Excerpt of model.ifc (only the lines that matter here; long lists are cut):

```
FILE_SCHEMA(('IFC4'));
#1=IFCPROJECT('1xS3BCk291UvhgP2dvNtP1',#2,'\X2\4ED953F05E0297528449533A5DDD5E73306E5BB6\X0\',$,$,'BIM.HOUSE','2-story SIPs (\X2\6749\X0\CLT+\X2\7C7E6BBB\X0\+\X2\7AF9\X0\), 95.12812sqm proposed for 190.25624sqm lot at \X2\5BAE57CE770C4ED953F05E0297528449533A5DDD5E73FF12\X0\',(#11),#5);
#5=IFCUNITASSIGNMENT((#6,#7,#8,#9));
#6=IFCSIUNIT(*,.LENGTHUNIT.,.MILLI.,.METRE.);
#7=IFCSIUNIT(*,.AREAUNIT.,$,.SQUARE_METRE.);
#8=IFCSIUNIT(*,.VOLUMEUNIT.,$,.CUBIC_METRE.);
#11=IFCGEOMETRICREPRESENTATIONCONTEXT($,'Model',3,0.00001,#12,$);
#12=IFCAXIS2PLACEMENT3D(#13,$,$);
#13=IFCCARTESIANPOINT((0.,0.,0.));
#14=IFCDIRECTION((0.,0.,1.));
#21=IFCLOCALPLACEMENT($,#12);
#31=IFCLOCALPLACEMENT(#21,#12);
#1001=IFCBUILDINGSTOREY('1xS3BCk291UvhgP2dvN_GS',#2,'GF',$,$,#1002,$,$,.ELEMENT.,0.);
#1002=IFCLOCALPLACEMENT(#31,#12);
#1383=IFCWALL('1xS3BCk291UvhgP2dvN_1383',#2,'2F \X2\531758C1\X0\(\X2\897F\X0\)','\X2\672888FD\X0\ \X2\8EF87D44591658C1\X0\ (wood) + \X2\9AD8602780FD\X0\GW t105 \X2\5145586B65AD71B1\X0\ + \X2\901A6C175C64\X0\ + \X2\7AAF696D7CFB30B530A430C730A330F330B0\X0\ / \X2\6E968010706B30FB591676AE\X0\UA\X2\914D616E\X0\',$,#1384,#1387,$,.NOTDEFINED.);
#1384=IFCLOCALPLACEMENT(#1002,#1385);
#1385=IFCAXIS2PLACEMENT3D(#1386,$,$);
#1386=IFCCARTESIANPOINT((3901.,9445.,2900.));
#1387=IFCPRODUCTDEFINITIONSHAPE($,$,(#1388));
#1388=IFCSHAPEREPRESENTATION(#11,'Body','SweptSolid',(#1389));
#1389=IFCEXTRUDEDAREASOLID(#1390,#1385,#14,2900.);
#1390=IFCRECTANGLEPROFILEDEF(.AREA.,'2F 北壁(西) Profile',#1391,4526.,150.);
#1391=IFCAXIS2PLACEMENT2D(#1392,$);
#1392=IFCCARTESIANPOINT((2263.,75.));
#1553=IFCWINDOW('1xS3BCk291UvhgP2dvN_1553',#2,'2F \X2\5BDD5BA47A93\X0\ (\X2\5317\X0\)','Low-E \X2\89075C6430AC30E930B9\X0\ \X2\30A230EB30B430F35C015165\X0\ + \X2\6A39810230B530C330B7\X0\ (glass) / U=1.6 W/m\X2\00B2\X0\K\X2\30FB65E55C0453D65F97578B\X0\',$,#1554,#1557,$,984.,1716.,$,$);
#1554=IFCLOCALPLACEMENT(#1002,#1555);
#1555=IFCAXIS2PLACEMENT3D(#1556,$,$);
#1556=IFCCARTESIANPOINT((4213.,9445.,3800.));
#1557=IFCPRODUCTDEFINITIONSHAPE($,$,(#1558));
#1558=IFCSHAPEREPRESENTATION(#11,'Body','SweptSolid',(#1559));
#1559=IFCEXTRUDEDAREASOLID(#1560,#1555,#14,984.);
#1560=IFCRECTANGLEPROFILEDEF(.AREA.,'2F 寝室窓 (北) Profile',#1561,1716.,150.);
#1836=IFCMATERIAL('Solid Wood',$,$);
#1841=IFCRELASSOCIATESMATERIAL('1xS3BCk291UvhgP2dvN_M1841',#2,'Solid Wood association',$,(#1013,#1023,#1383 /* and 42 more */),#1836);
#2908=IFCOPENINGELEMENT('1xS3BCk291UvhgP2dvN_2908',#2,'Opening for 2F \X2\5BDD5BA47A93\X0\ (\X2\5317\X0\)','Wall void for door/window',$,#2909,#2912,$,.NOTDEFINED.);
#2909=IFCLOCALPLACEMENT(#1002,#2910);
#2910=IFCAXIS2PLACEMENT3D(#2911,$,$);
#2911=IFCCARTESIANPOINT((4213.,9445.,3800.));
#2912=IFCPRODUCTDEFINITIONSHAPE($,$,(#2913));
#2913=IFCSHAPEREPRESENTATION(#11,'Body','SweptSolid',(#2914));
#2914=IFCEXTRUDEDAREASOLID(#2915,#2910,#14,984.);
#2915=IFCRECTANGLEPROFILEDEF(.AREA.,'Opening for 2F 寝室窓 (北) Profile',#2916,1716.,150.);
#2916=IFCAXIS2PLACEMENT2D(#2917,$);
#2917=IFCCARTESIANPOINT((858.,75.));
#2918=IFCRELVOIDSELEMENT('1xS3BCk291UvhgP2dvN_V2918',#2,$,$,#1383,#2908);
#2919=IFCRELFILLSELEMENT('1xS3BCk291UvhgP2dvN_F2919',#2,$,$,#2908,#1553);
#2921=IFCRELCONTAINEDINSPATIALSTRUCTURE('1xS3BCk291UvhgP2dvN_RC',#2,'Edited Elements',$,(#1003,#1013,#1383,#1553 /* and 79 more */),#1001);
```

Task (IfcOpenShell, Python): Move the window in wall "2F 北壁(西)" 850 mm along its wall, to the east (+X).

```python
import ifcopenshell
import ifcopenshell.api.geometry
import ifcopenshell.util.placement

model = ifcopenshell.open("model.ifc")

window = model.by_id(1553)
opening = window.FillsVoids[0].RelatingOpeningElement
wall = opening.VoidsElements[0].RelatingBuildingElement

wall_matrix = ifcopenshell.util.placement.get_local_placement(wall.ObjectPlacement)
shift = wall_matrix[:3, 0] * 850.0
before = ifcopenshell.util.placement.get_local_placement(window.ObjectPlacement)[:3, 3].copy()

# The window is not placed relative to its opening, so move both.
for product in (opening, window):
    matrix = ifcopenshell.util.placement.get_local_placement(product.ObjectPlacement)
    matrix[:3, 3] += shift
    ifcopenshell.api.geometry.edit_object_placement(model, product=product, matrix=matrix, is_si=False)

after = ifcopenshell.util.placement.get_local_placement(window.ObjectPlacement)[:3, 3]
print("window moved by", (after - before).round(3) + 0.0)

model.write("model_edited.ifc")
```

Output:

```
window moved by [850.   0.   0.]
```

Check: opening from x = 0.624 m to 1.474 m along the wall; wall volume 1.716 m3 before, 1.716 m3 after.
